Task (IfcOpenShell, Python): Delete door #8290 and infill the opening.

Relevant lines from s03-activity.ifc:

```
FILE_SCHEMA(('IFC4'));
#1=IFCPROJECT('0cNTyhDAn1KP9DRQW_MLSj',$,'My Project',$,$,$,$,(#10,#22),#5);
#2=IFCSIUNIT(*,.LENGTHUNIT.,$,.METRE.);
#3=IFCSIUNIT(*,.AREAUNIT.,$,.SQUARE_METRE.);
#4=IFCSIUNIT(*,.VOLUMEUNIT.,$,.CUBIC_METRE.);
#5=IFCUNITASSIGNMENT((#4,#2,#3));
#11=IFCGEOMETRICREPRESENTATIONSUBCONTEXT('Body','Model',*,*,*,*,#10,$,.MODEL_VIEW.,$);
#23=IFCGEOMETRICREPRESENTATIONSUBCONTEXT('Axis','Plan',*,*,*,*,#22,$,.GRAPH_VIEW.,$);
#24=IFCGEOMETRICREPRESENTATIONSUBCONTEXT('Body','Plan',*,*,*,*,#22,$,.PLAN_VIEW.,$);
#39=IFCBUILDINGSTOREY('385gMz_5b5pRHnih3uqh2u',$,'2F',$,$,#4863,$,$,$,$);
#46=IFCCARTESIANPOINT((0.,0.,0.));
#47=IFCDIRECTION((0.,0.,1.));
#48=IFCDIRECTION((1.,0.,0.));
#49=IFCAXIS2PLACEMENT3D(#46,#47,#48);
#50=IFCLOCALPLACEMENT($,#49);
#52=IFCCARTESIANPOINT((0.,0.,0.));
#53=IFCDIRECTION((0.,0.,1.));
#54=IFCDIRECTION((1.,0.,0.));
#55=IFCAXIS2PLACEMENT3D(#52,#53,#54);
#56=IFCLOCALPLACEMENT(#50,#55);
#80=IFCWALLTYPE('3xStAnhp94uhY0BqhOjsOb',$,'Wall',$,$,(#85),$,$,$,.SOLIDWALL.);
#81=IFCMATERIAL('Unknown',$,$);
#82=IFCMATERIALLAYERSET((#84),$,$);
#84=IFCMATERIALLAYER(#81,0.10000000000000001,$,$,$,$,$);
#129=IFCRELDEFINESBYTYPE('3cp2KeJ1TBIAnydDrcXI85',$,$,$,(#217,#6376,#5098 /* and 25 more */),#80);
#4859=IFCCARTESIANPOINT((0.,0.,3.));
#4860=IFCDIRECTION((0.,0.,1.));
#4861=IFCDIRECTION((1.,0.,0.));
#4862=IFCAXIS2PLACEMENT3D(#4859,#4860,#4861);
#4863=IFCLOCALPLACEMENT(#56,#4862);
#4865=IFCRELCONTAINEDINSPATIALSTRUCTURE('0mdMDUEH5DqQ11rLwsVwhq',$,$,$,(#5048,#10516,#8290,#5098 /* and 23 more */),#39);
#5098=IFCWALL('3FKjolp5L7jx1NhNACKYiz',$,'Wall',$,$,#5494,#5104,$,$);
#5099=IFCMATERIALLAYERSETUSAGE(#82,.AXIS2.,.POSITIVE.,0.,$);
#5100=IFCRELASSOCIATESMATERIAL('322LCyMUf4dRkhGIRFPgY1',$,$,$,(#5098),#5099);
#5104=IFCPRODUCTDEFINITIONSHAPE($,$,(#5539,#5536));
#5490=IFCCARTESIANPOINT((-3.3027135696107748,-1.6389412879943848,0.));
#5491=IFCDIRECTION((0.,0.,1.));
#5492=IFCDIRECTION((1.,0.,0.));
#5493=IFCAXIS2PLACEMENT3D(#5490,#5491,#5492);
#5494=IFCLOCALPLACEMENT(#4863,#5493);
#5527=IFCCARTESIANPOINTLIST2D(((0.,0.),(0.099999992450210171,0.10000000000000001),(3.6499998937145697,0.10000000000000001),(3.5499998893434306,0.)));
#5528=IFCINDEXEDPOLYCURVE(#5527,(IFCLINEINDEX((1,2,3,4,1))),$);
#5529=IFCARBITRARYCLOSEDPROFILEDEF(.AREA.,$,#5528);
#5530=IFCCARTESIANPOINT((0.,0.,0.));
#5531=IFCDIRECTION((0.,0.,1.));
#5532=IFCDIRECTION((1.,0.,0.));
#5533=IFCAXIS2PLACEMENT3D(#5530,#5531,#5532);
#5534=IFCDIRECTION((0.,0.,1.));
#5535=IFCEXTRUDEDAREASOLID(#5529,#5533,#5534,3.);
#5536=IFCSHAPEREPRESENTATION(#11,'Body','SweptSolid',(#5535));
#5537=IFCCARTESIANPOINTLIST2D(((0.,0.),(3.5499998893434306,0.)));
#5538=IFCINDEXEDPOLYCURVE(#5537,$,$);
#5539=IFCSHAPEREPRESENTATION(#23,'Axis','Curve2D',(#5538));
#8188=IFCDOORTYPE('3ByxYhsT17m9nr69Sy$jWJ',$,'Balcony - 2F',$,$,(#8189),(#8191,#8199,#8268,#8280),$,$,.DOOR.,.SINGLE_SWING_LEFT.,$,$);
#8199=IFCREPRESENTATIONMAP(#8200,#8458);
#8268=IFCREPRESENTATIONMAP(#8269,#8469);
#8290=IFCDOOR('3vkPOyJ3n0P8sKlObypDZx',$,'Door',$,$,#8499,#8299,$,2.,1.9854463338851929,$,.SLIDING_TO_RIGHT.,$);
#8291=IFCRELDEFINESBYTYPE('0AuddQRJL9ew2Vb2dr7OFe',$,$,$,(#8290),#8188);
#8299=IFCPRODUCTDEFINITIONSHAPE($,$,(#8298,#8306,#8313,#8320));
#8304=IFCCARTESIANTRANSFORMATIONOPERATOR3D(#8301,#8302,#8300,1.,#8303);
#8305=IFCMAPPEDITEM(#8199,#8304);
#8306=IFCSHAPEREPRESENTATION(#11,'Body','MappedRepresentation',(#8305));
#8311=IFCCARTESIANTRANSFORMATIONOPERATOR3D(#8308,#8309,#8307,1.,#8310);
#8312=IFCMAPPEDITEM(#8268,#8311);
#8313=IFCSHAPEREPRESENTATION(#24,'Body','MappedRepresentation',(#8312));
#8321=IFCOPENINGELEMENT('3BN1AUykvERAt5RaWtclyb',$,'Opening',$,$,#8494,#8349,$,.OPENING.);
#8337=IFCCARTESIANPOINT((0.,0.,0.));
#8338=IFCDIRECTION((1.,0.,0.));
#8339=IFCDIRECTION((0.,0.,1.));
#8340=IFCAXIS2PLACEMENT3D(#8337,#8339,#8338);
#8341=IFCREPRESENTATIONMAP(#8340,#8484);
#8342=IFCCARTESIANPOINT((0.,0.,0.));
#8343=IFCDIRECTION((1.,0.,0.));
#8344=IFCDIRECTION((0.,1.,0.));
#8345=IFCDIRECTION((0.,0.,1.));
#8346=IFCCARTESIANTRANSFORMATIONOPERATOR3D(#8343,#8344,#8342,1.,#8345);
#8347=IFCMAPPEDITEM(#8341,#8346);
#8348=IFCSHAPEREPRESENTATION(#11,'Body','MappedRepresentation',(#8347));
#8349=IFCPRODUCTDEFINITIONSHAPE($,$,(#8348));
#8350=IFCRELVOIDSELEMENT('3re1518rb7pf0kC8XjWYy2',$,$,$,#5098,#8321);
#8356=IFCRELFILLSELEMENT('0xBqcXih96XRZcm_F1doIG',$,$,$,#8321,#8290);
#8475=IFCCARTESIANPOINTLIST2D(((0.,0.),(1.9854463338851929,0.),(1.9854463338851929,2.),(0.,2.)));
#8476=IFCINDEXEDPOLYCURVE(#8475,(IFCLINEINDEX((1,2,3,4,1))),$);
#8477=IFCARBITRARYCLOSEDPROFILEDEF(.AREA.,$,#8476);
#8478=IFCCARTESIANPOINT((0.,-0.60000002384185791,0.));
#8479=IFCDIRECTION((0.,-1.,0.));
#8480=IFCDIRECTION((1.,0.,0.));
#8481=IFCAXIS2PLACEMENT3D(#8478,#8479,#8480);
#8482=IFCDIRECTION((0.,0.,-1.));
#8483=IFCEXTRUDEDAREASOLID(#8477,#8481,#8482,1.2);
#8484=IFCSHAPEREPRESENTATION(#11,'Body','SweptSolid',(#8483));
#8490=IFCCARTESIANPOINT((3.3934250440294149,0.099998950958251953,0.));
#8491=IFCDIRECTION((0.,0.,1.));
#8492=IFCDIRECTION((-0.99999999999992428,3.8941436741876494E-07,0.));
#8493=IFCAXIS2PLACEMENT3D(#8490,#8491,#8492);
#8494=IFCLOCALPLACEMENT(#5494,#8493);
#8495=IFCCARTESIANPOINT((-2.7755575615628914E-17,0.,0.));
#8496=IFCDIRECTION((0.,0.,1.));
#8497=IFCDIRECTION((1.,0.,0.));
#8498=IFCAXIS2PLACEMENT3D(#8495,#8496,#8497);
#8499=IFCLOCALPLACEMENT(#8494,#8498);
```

```python
import ifcopenshell
import ifcopenshell.api.feature
import ifcopenshell.api.root
import ifcopenshell.geom
import ifcopenshell.util.shape

model = ifcopenshell.open("s03-activity.ifc")
settings = ifcopenshell.geom.settings()


def volume(element):
    """Net volume in cubic metres, openings subtracted."""
    shape = ifcopenshell.geom.create_shape(settings, element)
    return ifcopenshell.util.shape.get_volume(shape.geometry)


door = model.by_id(8290)
opening = door.FillsVoids[0].RelatingOpeningElement
wall = opening.VoidsElements[0].RelatingBuildingElement
before = volume(wall)

ifcopenshell.api.root.remove_product(model, product=door)
ifcopenshell.api.feature.remove_feature(model, feature=opening)

after = volume(wall)

print(f"wall volume {before:.3f} -> {after:.3f} m3")

model.write("s03-activity_rev.ifc")
```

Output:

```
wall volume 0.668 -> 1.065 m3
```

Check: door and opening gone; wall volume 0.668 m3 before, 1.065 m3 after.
